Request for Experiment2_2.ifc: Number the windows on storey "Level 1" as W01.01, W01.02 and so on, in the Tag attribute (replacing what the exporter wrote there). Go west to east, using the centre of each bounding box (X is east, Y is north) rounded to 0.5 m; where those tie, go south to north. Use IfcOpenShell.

First a look at what the model holds.

```python
import ifcopenshell
import ifcopenshell.util.element
import ifcopenshell.util.placement

model = ifcopenshell.open("Experiment2_2.ifc")
print(model.schema)
storey = next(s for s in model.by_type("IfcBuildingStorey") if s.Name == "Level 1")
windows = [e for e in ifcopenshell.util.element.get_decomposition(storey) if e.is_a("IfcWindow")]
for e in sorted(windows, key=lambda e: e.id()):
    origin = ifcopenshell.util.placement.get_local_placement(e.ObjectPlacement)[:3, 3]
    print(e.id(), e.Tag, e.Name, origin.round(2) + 0.0, sep=" | ")
```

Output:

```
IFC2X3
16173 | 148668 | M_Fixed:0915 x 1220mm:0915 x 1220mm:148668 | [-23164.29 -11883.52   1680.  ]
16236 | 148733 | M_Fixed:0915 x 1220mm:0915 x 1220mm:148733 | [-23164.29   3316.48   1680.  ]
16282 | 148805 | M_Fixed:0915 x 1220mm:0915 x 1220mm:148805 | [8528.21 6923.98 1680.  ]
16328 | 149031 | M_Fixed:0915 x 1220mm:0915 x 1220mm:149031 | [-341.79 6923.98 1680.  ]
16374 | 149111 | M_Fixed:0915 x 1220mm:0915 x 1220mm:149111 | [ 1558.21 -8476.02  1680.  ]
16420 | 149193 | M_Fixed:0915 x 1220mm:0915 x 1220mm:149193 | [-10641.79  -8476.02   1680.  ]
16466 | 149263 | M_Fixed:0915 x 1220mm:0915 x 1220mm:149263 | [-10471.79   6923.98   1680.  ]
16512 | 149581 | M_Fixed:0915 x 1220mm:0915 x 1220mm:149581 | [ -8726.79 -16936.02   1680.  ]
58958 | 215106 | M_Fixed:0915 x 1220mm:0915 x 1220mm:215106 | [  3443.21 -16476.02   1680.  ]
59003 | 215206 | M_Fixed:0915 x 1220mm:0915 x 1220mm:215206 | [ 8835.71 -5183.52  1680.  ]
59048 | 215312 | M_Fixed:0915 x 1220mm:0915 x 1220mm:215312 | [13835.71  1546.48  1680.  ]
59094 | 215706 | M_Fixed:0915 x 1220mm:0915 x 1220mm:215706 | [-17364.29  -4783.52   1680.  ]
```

```python
import ifcopenshell
import ifcopenshell.geom
import ifcopenshell.util.element
import ifcopenshell.util.shape

model = ifcopenshell.open("Experiment2_2.ifc")
settings = ifcopenshell.geom.settings()
settings.set("use-world-coords", True)


def centre(element):
    shape = ifcopenshell.geom.create_shape(settings, element)
    return ifcopenshell.util.shape.get_bbox_centroid(shape.geometry)


storey = next(s for s in model.by_type("IfcBuildingStorey") if s.Name == "Level 1")
windows = [e for e in ifcopenshell.util.element.get_decomposition(storey) if e.is_a("IfcWindow")]

# Insertion points can sit at a corner or the storey origin, so sort by the geometry (in metres).
centres = {e: centre(e) for e in windows}
windows.sort(key=lambda e: (round(centres[e][0] / 0.5), centres[e][1]))

for i, e in enumerate(windows, start=1):
    number = f"W01.{i:02d}"
    e.Tag = number
    print(e.id(), number)

model.write("Experiment2_2-out.ifc")
```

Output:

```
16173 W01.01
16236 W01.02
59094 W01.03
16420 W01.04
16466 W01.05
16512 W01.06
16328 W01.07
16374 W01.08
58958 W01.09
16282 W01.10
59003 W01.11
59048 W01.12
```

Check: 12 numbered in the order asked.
